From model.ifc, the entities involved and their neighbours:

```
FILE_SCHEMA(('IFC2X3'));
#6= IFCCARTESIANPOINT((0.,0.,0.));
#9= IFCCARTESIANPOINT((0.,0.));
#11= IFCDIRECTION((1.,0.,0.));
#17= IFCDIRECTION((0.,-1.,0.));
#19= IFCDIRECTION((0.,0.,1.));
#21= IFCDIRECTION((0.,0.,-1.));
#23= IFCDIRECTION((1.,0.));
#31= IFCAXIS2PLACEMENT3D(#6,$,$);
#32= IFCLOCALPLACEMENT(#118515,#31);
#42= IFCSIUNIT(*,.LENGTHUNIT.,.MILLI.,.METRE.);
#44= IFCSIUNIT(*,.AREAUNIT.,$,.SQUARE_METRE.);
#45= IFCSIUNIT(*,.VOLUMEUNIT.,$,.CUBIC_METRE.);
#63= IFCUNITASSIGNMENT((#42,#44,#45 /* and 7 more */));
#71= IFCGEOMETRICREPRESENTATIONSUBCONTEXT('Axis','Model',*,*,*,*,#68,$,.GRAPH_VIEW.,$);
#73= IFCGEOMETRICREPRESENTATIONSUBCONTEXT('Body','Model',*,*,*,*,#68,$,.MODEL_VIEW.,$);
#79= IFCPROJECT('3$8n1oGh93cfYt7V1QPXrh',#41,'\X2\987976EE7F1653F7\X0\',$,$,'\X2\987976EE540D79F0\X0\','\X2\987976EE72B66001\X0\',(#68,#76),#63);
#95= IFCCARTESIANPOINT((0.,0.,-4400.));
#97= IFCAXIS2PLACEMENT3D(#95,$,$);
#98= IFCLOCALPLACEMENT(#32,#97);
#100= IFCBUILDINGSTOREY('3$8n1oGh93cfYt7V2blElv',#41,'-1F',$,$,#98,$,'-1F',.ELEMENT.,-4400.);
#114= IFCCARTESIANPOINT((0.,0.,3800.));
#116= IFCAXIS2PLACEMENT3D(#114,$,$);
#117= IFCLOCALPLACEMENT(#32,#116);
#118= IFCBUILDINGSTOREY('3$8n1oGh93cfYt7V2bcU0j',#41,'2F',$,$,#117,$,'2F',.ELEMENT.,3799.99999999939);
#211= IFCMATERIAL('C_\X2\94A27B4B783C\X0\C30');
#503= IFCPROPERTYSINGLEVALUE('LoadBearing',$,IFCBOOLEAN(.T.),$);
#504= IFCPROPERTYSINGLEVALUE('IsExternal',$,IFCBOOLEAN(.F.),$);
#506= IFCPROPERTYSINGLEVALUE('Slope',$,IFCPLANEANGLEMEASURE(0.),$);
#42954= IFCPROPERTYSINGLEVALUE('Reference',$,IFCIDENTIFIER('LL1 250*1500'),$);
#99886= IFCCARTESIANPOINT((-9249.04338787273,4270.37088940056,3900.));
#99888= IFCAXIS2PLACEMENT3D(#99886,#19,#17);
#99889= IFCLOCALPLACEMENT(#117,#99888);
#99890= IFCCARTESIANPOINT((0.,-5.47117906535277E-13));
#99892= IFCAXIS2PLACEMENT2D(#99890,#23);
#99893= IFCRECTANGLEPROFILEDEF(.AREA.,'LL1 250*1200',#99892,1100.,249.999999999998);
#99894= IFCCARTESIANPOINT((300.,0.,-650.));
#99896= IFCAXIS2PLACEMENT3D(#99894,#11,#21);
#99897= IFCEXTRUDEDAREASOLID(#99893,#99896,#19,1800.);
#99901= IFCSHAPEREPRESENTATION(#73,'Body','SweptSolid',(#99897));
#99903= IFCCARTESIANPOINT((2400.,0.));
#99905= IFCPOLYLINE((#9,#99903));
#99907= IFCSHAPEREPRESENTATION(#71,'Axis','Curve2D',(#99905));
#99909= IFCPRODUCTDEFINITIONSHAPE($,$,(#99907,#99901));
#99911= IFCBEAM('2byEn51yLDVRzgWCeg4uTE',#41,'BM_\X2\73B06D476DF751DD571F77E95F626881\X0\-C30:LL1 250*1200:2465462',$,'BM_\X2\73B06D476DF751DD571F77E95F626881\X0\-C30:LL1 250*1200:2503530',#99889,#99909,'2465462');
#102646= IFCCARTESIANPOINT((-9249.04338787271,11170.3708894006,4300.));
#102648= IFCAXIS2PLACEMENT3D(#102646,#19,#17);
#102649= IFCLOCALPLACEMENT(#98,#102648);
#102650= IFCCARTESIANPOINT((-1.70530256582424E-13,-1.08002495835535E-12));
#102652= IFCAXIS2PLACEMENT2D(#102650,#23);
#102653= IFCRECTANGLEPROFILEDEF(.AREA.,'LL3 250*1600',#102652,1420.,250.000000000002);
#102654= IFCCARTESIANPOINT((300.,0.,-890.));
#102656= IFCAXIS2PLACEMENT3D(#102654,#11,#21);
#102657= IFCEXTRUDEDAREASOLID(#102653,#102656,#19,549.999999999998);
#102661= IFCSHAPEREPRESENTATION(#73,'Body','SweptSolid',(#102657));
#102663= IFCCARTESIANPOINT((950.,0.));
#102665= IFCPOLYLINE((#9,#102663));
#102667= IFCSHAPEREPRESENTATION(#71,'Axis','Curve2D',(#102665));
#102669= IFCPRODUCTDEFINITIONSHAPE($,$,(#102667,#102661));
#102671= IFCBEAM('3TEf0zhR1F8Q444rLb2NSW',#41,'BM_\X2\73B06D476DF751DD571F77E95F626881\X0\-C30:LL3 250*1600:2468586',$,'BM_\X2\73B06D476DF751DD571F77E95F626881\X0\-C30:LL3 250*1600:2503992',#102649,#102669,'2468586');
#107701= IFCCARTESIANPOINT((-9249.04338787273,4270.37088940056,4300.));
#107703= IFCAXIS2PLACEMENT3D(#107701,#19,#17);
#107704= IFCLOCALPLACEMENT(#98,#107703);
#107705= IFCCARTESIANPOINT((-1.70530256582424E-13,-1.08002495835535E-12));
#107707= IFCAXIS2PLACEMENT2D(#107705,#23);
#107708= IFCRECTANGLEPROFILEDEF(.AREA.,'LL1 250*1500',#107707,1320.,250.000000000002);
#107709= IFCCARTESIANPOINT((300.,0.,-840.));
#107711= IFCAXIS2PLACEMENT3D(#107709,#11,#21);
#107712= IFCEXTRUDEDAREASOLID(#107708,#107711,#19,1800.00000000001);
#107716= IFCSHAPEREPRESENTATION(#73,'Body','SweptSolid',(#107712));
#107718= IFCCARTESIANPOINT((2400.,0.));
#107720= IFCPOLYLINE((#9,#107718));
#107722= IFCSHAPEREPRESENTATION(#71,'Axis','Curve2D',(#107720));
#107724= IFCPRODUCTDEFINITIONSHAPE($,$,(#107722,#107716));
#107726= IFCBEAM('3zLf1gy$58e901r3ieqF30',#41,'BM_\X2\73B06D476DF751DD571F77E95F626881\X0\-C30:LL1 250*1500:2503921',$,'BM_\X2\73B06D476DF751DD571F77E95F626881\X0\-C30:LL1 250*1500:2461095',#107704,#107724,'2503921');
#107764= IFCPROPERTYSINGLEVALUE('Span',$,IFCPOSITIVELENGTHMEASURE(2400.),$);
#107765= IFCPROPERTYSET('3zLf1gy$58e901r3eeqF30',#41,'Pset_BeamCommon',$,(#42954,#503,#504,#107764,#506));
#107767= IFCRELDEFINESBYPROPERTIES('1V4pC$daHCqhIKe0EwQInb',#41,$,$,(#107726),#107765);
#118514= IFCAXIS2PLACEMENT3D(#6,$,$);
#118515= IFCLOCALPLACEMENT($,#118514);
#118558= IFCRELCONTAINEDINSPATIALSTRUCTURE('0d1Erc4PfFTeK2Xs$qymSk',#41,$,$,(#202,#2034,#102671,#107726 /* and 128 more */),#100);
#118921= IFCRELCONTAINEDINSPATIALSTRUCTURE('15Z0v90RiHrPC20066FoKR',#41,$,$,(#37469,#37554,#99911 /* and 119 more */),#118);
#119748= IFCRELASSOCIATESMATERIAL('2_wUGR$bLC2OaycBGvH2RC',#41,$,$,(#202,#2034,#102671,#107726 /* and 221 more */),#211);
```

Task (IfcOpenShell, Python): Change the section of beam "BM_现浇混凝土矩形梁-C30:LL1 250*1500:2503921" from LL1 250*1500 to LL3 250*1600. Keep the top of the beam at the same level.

```python
import ifcopenshell
import ifcopenshell.api.pset
import ifcopenshell.util.element
import ifcopenshell.util.representation

model = ifcopenshell.open("model.ifc")

member = model.by_guid("3zLf1gy$58e901r3ieqF30")
source = next(p for p in model.by_type("IfcRectangleProfileDef") if p.ProfileName == "LL3 250*1600")

body = ifcopenshell.util.representation.get_representation(member, "Model", "Body")
solid = body.Items[0]
old_profile = solid.SweptArea

# Copy the section's sizes but keep this member's own profile position.
profile = ifcopenshell.util.element.copy(model, source)
# Profiles are centred, so shift by half the change in depth to hold the top.
shift = (old_profile.XDim - profile.XDim) / 2
x, y = old_profile.Position.Location.Coordinates
up = (-1.0, 0.0)  # upwards, in the solid's own plane
location = model.createIfcCartesianPoint((x + up[0] * shift, y + up[1] * shift))
profile.Position = model.createIfcAxis2Placement2D(location, old_profile.Position.RefDirection)
solid.SweptArea = profile
if not model.get_total_inverses(old_profile):
    ifcopenshell.util.element.remove_deep2(model, old_profile)
member.Name = member.Name.replace("LL1 250*1500", "LL3 250*1600")
member.ObjectType = member.ObjectType.replace("LL1 250*1500", "LL3 250*1600")
pset = model.by_id(ifcopenshell.util.element.get_pset(member, "Pset_BeamCommon", should_inherit=False)["id"])
ifcopenshell.api.pset.edit_pset(model, pset=pset, properties={"Reference": "LL3 250*1600"})

print(solid.SweptArea)

model.write("model_updated.ifc")
```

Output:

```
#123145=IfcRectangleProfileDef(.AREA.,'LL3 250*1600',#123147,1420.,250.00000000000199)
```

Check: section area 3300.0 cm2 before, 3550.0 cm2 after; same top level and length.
